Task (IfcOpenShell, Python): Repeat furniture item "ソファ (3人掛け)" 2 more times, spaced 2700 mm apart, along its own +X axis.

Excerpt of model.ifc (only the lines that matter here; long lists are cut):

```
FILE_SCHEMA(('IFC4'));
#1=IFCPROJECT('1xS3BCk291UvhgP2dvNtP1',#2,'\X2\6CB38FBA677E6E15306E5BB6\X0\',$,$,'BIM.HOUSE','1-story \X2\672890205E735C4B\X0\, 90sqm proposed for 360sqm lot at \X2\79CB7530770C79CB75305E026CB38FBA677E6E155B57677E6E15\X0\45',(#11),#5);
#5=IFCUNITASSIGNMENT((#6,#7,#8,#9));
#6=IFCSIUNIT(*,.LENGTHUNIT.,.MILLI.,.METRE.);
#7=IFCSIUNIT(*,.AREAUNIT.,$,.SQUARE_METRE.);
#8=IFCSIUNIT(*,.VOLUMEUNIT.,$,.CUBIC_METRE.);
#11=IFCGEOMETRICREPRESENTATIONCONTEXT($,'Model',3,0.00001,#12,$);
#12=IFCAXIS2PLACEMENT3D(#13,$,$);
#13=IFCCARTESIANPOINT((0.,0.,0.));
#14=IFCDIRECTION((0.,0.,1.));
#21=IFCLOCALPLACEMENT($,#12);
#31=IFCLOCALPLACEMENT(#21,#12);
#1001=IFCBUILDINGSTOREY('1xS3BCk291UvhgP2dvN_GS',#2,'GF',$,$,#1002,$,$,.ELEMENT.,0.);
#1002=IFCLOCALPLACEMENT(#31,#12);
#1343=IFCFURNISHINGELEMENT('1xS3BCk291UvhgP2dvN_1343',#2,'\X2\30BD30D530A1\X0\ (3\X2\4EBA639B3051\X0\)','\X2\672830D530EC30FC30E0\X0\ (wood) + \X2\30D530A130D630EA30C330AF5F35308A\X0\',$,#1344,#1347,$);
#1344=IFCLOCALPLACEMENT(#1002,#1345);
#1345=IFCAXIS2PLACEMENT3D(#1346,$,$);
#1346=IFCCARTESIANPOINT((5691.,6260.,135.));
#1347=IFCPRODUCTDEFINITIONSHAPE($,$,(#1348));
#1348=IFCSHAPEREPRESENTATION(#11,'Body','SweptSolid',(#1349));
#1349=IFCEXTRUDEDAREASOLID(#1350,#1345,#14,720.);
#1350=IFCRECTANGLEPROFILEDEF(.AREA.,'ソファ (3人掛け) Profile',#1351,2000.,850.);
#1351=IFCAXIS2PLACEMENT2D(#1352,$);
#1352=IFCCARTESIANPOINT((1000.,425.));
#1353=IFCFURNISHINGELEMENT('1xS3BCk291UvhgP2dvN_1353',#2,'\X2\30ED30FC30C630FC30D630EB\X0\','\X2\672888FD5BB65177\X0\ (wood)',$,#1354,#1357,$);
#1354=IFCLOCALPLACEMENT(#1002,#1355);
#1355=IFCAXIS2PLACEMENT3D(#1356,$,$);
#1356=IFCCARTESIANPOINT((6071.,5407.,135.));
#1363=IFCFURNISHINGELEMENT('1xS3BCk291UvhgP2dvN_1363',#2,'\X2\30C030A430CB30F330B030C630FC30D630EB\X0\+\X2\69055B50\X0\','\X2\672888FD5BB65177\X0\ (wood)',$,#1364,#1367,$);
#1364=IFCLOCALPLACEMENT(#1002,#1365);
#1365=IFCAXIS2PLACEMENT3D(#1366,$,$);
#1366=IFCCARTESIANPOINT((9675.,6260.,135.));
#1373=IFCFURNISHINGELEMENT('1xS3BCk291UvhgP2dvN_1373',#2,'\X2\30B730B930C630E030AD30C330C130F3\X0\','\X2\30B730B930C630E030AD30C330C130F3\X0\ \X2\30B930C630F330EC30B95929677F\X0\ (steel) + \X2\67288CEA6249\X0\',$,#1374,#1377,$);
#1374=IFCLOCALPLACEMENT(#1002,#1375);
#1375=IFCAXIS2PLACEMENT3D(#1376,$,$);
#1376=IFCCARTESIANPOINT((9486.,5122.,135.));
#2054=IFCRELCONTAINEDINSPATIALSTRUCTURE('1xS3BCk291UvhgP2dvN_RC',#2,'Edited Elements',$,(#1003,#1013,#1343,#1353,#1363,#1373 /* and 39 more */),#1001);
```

```python
import ifcopenshell
import ifcopenshell.api.geometry
import ifcopenshell.api.root
import ifcopenshell.util.element
import ifcopenshell.util.placement

model = ifcopenshell.open("model.ifc")


def reuse_history(source, copy):
    """copy_class also copies each property set's owner history, people and application; keep the originals."""
    for rel in copy.IsDefinedBy:
        if rel.is_a("IfcRelDefinesByProperties") and (history := rel.RelatingPropertyDefinition.OwnerHistory):
            rel.RelatingPropertyDefinition.OwnerHistory = source.OwnerHistory
            ifcopenshell.util.element.remove_deep2(model, history)


source = model.by_id(1343)
base = ifcopenshell.util.placement.get_local_placement(source.ObjectPlacement)
step = base[:3, 0] * 2700.0

for i in range(1, 3):
    copy = ifcopenshell.api.root.copy_class(model, product=source)
    copy.Representation = ifcopenshell.util.element.copy_deep(
        model, source.Representation, exclude=["IfcGeometricRepresentationContext", "IfcRepresentationMap"]
    )
    reuse_history(source, copy)
    matrix = base.copy()
    matrix[:3, 3] += i * step
    print("added at", matrix[:3, 3].round(3) + 0.0)
    ifcopenshell.api.geometry.edit_object_placement(model, product=copy, matrix=matrix, is_si=False)

model.write("model_edited.ifc")
```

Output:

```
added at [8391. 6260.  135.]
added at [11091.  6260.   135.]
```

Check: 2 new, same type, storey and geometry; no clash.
